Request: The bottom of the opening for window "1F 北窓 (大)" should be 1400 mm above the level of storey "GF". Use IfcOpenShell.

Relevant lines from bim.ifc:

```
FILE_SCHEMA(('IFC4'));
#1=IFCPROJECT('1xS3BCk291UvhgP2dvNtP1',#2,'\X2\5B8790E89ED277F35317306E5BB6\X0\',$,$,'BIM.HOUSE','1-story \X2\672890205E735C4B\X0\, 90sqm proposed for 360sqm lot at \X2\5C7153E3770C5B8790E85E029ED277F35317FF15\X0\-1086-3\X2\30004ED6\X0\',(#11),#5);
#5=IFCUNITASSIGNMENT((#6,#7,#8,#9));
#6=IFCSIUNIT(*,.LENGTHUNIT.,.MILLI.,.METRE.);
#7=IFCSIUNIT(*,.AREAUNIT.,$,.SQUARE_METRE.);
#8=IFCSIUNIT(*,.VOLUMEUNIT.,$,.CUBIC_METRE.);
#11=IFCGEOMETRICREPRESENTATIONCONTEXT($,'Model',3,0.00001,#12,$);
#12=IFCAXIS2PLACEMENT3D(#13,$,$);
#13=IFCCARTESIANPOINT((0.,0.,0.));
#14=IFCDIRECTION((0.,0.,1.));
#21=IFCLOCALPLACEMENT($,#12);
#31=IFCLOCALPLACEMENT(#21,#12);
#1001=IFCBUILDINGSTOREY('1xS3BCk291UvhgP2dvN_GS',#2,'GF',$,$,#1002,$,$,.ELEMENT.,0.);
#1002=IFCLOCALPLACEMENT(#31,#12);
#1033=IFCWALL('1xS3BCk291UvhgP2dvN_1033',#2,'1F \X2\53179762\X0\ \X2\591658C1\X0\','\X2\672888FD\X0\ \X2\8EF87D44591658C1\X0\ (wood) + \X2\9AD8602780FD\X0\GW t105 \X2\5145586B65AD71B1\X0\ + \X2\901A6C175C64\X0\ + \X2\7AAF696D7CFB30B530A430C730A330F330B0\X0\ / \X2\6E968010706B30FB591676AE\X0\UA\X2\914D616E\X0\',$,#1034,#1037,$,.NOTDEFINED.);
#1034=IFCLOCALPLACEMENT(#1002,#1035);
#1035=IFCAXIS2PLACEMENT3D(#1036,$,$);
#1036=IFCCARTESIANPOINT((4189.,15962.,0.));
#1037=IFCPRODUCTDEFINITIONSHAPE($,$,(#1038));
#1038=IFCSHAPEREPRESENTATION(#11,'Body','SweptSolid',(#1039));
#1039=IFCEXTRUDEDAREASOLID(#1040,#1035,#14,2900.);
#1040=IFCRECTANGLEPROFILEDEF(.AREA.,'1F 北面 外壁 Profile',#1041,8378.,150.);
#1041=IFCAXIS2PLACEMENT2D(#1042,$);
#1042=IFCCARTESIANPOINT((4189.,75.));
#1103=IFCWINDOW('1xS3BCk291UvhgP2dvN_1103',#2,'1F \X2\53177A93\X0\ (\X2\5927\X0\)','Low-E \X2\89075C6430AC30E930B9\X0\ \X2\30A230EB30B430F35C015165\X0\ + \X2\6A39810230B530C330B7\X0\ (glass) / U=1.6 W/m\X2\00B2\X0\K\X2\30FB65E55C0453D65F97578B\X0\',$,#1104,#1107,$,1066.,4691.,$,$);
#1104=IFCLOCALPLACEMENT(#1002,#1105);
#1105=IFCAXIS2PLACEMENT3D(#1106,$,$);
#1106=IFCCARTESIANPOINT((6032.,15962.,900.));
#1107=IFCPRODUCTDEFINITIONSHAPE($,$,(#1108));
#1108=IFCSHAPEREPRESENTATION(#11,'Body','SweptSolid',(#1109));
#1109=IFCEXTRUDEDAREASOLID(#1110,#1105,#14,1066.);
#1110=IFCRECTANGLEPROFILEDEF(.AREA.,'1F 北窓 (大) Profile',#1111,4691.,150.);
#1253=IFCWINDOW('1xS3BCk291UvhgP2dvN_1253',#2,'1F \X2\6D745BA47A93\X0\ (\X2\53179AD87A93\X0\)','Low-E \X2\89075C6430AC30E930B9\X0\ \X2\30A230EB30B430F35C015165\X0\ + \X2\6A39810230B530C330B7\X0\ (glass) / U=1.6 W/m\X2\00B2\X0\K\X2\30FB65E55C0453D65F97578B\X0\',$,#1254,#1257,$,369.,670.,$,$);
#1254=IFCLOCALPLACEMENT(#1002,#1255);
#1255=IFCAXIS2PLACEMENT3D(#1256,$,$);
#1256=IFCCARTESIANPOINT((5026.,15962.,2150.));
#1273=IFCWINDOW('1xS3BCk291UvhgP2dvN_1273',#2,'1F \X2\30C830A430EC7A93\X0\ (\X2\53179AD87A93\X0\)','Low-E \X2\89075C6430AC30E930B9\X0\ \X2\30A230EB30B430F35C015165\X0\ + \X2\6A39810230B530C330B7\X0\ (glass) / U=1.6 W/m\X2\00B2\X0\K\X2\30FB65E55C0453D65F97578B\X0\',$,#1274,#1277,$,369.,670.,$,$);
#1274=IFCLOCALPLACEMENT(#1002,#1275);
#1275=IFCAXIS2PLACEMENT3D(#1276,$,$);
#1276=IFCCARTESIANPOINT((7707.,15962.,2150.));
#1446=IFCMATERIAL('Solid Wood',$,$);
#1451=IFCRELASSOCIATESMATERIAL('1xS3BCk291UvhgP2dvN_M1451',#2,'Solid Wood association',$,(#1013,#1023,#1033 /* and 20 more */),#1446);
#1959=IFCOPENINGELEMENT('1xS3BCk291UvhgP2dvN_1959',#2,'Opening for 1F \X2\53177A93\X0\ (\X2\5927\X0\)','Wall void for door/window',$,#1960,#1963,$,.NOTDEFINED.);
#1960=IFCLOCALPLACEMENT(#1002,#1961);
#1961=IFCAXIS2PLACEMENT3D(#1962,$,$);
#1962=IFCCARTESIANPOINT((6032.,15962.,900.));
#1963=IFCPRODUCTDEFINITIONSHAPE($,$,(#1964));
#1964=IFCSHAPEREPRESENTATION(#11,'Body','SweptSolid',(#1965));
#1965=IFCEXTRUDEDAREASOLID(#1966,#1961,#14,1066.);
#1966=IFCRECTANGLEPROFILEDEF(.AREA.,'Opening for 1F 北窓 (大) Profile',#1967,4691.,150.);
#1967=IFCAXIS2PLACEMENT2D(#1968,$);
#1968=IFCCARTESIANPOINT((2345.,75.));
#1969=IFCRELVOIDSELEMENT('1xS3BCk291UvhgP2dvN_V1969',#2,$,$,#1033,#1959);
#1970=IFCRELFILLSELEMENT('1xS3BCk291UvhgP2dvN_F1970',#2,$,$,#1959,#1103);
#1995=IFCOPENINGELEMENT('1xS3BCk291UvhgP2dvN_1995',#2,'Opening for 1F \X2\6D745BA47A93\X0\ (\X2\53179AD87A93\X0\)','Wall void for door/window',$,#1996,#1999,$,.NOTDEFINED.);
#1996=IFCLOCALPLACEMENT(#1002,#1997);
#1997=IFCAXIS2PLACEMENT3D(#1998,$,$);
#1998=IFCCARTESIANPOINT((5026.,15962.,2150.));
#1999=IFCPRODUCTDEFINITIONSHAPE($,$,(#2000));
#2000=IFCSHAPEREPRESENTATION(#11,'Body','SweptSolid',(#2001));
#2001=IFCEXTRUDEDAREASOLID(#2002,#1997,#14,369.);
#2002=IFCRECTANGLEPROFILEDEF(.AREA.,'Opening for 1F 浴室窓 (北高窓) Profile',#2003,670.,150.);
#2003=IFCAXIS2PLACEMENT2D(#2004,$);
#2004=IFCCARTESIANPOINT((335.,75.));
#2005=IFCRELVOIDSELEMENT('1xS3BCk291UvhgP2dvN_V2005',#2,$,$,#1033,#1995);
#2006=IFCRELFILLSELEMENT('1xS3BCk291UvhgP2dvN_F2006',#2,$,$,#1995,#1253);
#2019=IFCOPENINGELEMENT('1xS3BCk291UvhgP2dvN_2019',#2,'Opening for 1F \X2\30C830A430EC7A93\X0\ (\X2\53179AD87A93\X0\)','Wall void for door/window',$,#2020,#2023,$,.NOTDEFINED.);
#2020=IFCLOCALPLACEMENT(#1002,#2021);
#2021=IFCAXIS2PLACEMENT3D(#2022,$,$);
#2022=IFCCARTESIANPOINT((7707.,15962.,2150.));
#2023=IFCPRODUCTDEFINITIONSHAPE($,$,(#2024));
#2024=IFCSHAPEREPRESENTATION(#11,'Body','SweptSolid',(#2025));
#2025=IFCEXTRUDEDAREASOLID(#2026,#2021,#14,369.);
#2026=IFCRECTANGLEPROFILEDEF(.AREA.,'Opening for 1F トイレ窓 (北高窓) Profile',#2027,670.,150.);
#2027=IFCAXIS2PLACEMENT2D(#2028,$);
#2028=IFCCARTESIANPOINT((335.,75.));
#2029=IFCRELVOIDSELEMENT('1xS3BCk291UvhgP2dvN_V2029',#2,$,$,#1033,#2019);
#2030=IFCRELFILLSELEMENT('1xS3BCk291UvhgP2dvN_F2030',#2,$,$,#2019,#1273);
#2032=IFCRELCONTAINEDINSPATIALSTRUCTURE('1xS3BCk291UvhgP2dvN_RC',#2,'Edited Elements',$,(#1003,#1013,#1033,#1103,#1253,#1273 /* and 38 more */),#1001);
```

```python
import numpy as np
import ifcopenshell
import ifcopenshell.api.geometry
import ifcopenshell.geom
import ifcopenshell.util.element
import ifcopenshell.util.placement
import ifcopenshell.util.shape
import ifcopenshell.util.unit

model = ifcopenshell.open("bim.ifc")
unit_scale = ifcopenshell.util.unit.calculate_unit_scale(model)

window = model.by_guid("1xS3BCk291UvhgP2dvN_1103")
opening = window.FillsVoids[0].RelatingOpeningElement
storey = ifcopenshell.util.element.get_container(window, ifc_class="IfcBuildingStorey")
level = ifcopenshell.util.placement.get_local_placement(storey.ObjectPlacement)[2, 3]

# The opening's origin need not be at the sill, so measure its lowest point.
shape = ifcopenshell.geom.create_shape(ifcopenshell.geom.settings(), opening)
bottom = ifcopenshell.util.shape.get_shape_bottom_elevation(shape, shape.geometry) / unit_scale
dz = level + 1.4 / unit_scale - bottom

shift = np.array([0.0, 0.0, dz])
# The window is not placed relative to its opening, so move both.
for product in (opening, window):
    matrix = ifcopenshell.util.placement.get_local_placement(product.ObjectPlacement)
    matrix[:3, 3] += shift
    ifcopenshell.api.geometry.edit_object_placement(model, product=product, matrix=matrix, is_si=False)

print(f"moved by {dz * unit_scale:+.3f} m")

model.write("bim_updated.ifc")
```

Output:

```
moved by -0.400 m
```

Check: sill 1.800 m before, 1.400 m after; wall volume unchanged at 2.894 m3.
